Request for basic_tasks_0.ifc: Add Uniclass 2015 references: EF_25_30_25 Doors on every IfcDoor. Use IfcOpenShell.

First a look at what the model holds.

```python
import ifcopenshell

model = ifcopenshell.open("basic_tasks_0.ifc")
print(model.schema)
print("classifications:", [c.Name for c in model.by_type("IfcClassification")])
for ifc_class in ("IfcDoor", "IfcRoof", "IfcStair", "IfcWall", "IfcWindow"):
    print(ifc_class, len(model.by_type(ifc_class)))
```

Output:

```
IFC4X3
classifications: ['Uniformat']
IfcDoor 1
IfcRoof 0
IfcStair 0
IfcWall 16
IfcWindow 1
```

```python
import ifcopenshell
import ifcopenshell.api.classification

model = ifcopenshell.open("basic_tasks_0.ifc")

system = ifcopenshell.api.classification.add_classification(model, classification="Uniclass 2015")

codes = {
    "IfcDoor": ("EF_25_30_25", "Doors"),
}
for ifc_class, (code, name) in codes.items():
    products = model.by_type(ifc_class)
    ifcopenshell.api.classification.add_reference(
        model, products=products, classification=system, identification=code, name=name
    )
    print(code, len(products))

model.write("basic_tasks_0_v2.ifc")
```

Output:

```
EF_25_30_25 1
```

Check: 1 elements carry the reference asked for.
